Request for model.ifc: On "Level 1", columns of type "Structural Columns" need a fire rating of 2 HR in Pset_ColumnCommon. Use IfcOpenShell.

First a look at what the model holds.

```python
import ifcopenshell
import ifcopenshell.util.element

model = ifcopenshell.open("model.ifc")
print(model.schema)
storey = next(s for s in model.by_type("IfcBuildingStorey") if s.Name == "Level 1")
columns = [e for e in ifcopenshell.util.element.get_decomposition(storey) if e.is_a("IfcColumn")]
seen = {}
for e in columns:
    element_type = ifcopenshell.util.element.get_type(e)
    key = (element_type.Name if element_type != e and element_type else None, ifcopenshell.util.element.get_pset(e, "Pset_ColumnCommon", "FireRating"))
    seen[key] = seen.get(key, 0) + 1
for (name, value), count in sorted(seen.items(), key=str):
    print(count, "x", name, "|", value)
```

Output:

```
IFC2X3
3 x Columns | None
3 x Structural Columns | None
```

```python
import ifcopenshell
import ifcopenshell.api.pset
import ifcopenshell.util.element

model = ifcopenshell.open("model.ifc")

storey = next(s for s in model.by_type("IfcBuildingStorey") if s.Name == "Level 1")
columns = [e for e in ifcopenshell.util.element.get_decomposition(storey) if e.is_a("IfcColumn")]

count = 0
for e in columns:
    element_type = ifcopenshell.util.element.get_type(e)
    if element_type in (None, e) or element_type.Name != "Structural Columns":
        continue
    # add_pset returns the element's existing set when there is one.
    pset = ifcopenshell.api.pset.add_pset(model, product=e, name="Pset_ColumnCommon")
    ifcopenshell.api.pset.edit_pset(model, pset=pset, properties={"FireRating": "2 HR"})
    count += 1

print(count, "columns updated")

model.write("model_rev.ifc")
```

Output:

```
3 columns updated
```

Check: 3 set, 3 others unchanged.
